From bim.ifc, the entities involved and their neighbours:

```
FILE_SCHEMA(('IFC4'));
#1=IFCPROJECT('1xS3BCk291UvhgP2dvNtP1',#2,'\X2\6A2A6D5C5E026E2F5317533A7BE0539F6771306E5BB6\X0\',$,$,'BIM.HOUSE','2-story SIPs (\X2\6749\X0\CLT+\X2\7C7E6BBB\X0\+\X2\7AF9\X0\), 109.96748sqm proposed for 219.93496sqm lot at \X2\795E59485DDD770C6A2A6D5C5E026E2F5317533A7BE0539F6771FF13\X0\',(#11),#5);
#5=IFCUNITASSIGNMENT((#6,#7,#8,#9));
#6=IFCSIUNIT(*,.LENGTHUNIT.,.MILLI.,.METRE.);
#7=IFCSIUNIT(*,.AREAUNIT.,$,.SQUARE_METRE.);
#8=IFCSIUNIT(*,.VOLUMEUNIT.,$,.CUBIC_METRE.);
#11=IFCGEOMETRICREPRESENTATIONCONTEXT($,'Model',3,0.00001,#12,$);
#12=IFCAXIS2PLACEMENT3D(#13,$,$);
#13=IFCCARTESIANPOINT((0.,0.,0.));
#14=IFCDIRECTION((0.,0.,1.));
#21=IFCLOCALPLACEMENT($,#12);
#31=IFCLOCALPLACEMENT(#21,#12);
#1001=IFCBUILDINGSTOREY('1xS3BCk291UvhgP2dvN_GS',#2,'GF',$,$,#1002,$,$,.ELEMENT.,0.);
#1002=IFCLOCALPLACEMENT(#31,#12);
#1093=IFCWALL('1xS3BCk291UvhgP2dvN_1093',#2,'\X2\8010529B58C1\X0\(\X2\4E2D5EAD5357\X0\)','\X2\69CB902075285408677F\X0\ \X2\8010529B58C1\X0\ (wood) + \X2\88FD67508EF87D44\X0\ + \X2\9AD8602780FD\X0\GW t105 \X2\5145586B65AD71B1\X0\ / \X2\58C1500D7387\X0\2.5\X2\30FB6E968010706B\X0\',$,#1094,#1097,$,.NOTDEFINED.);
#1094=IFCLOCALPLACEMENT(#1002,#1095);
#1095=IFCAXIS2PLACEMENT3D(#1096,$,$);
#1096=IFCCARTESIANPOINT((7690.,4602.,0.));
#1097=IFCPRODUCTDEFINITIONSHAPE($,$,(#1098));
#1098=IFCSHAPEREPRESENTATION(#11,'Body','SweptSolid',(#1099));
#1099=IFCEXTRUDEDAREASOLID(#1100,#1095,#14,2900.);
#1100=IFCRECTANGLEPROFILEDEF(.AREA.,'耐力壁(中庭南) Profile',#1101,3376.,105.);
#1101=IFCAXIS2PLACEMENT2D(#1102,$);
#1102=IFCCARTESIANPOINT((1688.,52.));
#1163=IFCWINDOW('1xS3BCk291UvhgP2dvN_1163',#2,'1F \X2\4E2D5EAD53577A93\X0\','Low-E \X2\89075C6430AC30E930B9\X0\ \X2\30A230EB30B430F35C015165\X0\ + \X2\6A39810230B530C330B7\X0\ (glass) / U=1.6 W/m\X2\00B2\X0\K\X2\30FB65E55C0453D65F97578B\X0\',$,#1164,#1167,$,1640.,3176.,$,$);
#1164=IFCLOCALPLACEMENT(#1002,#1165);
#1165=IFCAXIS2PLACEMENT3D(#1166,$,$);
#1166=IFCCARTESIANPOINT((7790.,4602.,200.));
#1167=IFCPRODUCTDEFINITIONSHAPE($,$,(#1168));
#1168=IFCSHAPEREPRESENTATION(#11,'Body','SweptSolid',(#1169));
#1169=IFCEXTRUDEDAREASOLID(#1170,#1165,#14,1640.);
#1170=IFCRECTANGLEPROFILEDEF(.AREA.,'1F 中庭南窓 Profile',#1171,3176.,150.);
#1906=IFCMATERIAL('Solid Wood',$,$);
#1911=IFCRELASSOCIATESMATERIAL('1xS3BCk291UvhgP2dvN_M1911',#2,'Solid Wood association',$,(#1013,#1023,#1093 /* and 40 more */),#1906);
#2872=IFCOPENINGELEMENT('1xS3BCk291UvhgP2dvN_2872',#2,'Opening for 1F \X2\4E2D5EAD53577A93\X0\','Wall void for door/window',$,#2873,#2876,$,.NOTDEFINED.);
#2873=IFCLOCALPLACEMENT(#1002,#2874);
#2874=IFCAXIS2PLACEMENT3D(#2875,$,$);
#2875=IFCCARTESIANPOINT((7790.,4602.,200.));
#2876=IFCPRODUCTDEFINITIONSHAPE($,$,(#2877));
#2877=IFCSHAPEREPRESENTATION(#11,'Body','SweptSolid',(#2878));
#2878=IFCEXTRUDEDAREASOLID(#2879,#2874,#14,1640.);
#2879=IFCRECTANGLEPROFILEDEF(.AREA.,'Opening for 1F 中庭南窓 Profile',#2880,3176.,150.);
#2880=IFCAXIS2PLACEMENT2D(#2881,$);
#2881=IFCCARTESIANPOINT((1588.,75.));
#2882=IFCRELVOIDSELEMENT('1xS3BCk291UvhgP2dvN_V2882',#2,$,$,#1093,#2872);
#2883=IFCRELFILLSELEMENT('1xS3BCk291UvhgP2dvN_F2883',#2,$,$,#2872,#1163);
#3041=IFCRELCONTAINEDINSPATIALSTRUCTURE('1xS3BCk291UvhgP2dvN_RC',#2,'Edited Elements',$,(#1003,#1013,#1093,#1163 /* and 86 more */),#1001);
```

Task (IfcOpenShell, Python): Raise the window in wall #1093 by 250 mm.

```python
import numpy as np
import ifcopenshell
import ifcopenshell.api.geometry
import ifcopenshell.util.placement
import ifcopenshell.util.unit

model = ifcopenshell.open("bim.ifc")
unit_scale = ifcopenshell.util.unit.calculate_unit_scale(model)

window = model.by_guid("1xS3BCk291UvhgP2dvN_1163")
opening = window.FillsVoids[0].RelatingOpeningElement
dz = 250.0

shift = np.array([0.0, 0.0, dz])
# The window is not placed relative to its opening, so move both.
for product in (opening, window):
    matrix = ifcopenshell.util.placement.get_local_placement(product.ObjectPlacement)
    matrix[:3, 3] += shift
    ifcopenshell.api.geometry.edit_object_placement(model, product=product, matrix=matrix, is_si=False)

print(f"moved by {dz * unit_scale:+.3f} m")

model.write("bim_updated.ifc")
```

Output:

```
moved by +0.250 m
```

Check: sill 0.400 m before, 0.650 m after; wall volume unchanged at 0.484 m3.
